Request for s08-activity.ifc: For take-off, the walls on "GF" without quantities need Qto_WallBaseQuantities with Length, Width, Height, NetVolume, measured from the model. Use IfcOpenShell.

First a look at what the model holds.

```python
import ifcopenshell
import ifcopenshell.util.element
import ifcopenshell.util.unit

model = ifcopenshell.open("s08-activity.ifc")
print(model.schema)
for unit_type in ("LENGTHUNIT", "AREAUNIT", "VOLUMEUNIT"):
    print(unit_type, ifcopenshell.util.unit.calculate_unit_scale(model, unit_type))
storey = next(s for s in model.by_type("IfcBuildingStorey") if s.Name == "GF")
walls = [e for e in ifcopenshell.util.element.get_decomposition(storey) if e.is_a("IfcWall")]
for e in sorted(walls, key=lambda e: e.id()):
    print(e.id(), e.is_a(), e.Name, list(ifcopenshell.util.element.get_psets(e, qtos_only=True)), sep=" | ")
```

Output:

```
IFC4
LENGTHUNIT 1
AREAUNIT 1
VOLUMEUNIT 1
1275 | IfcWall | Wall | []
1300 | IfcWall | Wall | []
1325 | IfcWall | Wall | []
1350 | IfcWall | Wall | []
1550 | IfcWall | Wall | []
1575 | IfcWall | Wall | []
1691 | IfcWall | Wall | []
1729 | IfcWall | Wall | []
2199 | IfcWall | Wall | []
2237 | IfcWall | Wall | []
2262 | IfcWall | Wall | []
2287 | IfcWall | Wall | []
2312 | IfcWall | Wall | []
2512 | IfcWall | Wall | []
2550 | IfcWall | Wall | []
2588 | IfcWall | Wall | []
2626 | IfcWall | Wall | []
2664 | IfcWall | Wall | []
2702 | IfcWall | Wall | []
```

```python
import ifcopenshell
import ifcopenshell.api.pset
import ifcopenshell.geom
import ifcopenshell.util.element
import ifcopenshell.util.shape
import ifcopenshell.util.unit

model = ifcopenshell.open("s08-activity.ifc")
unit_scale = ifcopenshell.util.unit.calculate_unit_scale(model)
volume_scale = ifcopenshell.util.unit.calculate_unit_scale(model, "VOLUMEUNIT")
settings = ifcopenshell.geom.settings()

storey = next(s for s in model.by_type("IfcBuildingStorey") if s.Name == "GF")
walls = [e for e in ifcopenshell.util.element.get_decomposition(storey) if e.is_a("IfcWall")]

for e in sorted(walls, key=lambda e: e.id()):
    if ifcopenshell.util.element.get_psets(e, qtos_only=True, should_inherit=False):
        continue
    # Geometry comes back in metres, in the element's own axes.
    shape = ifcopenshell.geom.create_shape(settings, e)
    values = {
        "Length": ifcopenshell.util.shape.get_x(shape.geometry) / unit_scale,
        "Width": ifcopenshell.util.shape.get_y(shape.geometry) / unit_scale,
        "Height": ifcopenshell.util.shape.get_z(shape.geometry) / unit_scale,
        "NetVolume": ifcopenshell.util.shape.get_volume(shape.geometry) / volume_scale,
    }
    qto = ifcopenshell.api.pset.add_qto(model, product=e, name="Qto_WallBaseQuantities")
    ifcopenshell.api.pset.edit_qto(model, qto=qto, properties=values)
    print(e.id(), {k: round(v, 3) for k, v in values.items()})

model.write("s08-activity_edited.ifc")
```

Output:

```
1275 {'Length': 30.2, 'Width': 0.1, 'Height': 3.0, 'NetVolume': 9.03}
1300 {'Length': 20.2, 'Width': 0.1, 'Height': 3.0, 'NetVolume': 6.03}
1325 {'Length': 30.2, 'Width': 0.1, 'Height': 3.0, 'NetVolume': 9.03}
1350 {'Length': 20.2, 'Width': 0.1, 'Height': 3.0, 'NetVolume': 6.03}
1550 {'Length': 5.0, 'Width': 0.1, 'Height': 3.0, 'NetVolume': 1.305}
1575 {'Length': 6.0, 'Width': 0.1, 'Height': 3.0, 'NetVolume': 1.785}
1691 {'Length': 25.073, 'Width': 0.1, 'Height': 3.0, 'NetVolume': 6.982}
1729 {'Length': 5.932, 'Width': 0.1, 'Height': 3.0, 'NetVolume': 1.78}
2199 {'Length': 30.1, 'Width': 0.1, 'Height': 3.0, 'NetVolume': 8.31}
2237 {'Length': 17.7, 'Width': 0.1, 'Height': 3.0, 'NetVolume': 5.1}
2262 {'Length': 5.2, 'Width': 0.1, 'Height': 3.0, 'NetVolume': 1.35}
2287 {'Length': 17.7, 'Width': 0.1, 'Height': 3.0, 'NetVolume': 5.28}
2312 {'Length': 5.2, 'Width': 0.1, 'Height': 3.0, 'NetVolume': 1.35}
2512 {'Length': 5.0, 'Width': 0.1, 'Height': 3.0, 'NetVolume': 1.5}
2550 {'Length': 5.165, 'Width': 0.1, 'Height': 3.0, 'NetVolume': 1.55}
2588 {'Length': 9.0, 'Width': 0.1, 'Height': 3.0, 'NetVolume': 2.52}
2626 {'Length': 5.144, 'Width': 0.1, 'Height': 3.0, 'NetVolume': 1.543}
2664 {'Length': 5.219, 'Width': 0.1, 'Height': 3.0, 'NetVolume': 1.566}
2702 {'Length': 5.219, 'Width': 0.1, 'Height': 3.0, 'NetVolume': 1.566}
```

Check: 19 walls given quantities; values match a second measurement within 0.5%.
